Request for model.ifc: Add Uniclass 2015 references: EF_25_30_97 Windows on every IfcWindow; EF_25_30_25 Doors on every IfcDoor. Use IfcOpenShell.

First a look at what the model holds.

```python
import ifcopenshell

model = ifcopenshell.open("model.ifc")
print(model.schema)
print("classifications:", [c.Name for c in model.by_type("IfcClassification")])
for ifc_class in ("IfcDoor", "IfcRoof", "IfcStair", "IfcWall", "IfcWindow"):
    print(ifc_class, len(model.by_type(ifc_class)))
```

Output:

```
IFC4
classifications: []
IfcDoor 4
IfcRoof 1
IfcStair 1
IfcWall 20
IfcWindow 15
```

```python
import ifcopenshell
import ifcopenshell.api.classification

model = ifcopenshell.open("model.ifc")

system = ifcopenshell.api.classification.add_classification(model, classification="Uniclass 2015")

codes = {
    "IfcWindow": ("EF_25_30_97", "Windows"),
    "IfcDoor": ("EF_25_30_25", "Doors"),
}
for ifc_class, (code, name) in codes.items():
    products = model.by_type(ifc_class)
    ifcopenshell.api.classification.add_reference(
        model, products=products, classification=system, identification=code, name=name
    )
    print(code, len(products))

model.write("model-out.ifc")
```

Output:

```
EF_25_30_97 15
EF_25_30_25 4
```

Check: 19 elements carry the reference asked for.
